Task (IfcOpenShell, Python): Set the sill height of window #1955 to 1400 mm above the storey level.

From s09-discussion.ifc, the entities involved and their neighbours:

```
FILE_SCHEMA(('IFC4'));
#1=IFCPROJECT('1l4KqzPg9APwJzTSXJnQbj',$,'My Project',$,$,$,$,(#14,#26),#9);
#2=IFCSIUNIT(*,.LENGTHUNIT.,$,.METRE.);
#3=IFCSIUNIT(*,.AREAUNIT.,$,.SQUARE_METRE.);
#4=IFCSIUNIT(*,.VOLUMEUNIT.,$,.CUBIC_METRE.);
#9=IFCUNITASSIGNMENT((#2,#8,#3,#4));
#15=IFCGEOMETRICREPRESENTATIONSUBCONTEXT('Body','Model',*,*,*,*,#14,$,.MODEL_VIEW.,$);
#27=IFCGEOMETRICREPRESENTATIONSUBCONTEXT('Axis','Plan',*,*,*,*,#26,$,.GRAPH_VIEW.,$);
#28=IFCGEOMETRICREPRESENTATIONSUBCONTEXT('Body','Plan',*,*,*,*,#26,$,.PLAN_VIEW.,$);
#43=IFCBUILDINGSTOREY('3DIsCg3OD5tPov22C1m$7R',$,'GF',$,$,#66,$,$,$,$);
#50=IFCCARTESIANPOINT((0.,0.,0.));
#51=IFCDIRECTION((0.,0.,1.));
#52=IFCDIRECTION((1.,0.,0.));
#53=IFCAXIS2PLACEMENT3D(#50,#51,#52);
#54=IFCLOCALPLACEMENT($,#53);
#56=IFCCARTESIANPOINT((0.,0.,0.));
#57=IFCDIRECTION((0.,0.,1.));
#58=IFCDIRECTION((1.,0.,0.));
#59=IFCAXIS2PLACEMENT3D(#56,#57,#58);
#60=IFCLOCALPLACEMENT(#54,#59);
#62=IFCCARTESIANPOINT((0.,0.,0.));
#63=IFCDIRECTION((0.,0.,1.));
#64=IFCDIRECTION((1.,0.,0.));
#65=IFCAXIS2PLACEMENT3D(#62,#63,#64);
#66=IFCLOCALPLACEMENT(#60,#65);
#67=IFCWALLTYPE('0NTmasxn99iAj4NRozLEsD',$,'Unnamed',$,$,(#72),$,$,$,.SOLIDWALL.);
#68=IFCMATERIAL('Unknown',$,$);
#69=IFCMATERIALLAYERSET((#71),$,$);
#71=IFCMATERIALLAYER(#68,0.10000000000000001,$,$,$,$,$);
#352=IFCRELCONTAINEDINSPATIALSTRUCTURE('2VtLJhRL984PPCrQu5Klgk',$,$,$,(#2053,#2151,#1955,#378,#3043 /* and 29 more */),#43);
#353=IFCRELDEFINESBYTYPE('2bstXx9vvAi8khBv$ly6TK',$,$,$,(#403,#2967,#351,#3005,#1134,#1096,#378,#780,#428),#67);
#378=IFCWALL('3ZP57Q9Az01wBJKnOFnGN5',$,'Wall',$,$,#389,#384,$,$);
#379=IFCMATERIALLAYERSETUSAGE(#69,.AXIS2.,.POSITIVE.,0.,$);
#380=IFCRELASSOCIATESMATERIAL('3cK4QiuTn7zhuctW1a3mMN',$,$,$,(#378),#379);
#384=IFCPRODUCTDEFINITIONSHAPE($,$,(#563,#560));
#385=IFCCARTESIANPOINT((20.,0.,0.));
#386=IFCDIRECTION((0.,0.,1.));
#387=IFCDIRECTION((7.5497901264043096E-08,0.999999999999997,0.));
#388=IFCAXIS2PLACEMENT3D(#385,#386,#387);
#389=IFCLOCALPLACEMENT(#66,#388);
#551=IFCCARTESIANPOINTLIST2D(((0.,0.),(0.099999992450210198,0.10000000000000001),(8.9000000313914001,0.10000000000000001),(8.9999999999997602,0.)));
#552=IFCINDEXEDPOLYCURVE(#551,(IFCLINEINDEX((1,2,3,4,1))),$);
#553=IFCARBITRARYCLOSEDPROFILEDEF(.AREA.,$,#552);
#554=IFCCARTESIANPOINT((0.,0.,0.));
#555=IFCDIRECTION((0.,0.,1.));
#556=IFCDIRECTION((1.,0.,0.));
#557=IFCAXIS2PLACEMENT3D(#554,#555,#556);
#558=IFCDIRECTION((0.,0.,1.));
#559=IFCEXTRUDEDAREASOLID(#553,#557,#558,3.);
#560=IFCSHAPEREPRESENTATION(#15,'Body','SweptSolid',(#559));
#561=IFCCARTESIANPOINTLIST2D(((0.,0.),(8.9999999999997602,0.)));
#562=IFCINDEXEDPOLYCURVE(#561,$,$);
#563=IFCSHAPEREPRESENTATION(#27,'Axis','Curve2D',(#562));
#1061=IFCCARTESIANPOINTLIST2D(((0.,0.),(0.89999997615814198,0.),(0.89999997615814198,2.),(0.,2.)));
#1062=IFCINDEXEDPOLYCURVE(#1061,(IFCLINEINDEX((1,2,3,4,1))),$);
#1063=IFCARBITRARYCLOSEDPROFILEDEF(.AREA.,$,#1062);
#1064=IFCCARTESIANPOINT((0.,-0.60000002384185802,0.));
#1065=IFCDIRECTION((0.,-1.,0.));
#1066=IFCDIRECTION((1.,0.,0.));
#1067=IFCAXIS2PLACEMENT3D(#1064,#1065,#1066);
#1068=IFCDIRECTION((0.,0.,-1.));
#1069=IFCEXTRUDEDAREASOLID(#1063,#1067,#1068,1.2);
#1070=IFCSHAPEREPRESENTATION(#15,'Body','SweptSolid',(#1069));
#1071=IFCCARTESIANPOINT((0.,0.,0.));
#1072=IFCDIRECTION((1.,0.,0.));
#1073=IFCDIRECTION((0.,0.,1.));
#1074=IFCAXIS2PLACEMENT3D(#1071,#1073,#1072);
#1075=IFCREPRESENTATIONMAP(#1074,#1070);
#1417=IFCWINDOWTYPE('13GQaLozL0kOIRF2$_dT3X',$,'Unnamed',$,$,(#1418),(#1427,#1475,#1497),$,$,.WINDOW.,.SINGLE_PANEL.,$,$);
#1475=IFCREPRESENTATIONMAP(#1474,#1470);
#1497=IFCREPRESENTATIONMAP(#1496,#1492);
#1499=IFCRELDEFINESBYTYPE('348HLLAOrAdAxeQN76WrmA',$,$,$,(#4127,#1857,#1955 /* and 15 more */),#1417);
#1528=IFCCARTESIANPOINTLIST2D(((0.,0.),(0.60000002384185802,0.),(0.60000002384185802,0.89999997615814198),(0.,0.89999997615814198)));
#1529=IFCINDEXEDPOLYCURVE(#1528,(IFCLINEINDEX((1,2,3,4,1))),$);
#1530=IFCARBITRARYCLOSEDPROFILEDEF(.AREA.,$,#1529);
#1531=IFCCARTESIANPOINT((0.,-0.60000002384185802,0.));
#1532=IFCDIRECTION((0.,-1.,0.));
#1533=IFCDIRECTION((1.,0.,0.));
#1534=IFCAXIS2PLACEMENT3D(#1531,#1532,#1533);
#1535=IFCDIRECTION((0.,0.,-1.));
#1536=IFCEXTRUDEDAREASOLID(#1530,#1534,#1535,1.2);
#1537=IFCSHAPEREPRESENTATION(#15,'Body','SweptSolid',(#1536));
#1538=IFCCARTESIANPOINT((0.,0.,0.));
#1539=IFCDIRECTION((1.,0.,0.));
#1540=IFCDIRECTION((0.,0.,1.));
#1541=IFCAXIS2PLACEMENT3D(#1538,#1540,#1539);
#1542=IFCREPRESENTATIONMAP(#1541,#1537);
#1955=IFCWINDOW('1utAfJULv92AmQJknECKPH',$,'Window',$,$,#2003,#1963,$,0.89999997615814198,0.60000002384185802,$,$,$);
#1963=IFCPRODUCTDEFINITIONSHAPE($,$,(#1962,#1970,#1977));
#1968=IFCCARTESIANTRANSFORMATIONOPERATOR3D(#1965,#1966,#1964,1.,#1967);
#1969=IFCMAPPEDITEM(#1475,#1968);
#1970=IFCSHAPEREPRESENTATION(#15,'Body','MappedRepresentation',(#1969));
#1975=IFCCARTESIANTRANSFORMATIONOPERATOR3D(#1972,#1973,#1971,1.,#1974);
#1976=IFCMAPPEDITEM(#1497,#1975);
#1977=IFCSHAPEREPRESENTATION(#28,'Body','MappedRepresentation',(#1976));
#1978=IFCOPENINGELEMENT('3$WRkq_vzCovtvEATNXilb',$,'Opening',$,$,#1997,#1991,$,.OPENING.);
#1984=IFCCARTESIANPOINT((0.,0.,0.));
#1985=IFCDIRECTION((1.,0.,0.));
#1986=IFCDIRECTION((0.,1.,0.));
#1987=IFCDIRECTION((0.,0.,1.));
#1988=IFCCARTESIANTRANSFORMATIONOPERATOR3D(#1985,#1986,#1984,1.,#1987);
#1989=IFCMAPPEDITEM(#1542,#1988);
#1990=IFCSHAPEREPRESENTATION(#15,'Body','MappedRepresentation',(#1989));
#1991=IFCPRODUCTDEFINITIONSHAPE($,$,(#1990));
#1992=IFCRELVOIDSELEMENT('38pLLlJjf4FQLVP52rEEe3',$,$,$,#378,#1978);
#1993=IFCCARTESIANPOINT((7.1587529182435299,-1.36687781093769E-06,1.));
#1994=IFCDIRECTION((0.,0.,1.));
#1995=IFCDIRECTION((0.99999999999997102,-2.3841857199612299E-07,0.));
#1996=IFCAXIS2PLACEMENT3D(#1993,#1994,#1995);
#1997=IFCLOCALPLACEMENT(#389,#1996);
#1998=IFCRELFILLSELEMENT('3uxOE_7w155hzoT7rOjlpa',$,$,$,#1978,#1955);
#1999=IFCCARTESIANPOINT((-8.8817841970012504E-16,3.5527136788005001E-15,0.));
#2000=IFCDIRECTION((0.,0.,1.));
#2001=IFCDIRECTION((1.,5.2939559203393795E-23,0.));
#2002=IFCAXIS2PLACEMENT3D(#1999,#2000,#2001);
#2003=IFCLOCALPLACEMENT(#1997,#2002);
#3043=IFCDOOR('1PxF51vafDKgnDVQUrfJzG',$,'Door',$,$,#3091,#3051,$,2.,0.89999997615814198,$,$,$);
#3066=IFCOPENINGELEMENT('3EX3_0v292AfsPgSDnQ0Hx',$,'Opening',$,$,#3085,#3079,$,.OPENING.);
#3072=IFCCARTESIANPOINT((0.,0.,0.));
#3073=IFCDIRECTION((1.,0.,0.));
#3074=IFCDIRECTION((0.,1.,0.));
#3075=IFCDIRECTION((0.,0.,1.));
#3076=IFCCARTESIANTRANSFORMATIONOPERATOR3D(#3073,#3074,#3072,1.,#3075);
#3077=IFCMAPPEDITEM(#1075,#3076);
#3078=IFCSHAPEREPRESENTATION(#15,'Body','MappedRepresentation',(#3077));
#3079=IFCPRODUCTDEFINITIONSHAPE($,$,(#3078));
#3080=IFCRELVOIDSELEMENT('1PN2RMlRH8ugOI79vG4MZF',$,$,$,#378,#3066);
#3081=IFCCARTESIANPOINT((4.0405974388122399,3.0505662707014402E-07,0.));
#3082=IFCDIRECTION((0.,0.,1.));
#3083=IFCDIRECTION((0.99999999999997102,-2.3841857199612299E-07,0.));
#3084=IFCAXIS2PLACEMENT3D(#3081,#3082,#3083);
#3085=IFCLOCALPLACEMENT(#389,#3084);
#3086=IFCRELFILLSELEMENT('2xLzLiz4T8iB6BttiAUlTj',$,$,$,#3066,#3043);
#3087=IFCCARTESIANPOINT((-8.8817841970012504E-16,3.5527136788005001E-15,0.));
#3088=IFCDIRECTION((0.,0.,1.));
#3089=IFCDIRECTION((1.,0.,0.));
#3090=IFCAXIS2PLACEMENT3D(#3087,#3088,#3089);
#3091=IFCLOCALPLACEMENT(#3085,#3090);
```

```python
import numpy as np
import ifcopenshell
import ifcopenshell.api.geometry
import ifcopenshell.geom
import ifcopenshell.util.element
import ifcopenshell.util.placement
import ifcopenshell.util.shape
import ifcopenshell.util.unit

model = ifcopenshell.open("s09-discussion.ifc")
unit_scale = ifcopenshell.util.unit.calculate_unit_scale(model)

window = model.by_guid("1utAfJULv92AmQJknECKPH")
opening = window.FillsVoids[0].RelatingOpeningElement
storey = ifcopenshell.util.element.get_container(window, ifc_class="IfcBuildingStorey")
level = ifcopenshell.util.placement.get_local_placement(storey.ObjectPlacement)[2, 3]

# The opening's origin need not be at the sill, so measure its lowest point.
shape = ifcopenshell.geom.create_shape(ifcopenshell.geom.settings(), opening)
bottom = ifcopenshell.util.shape.get_shape_bottom_elevation(shape, shape.geometry) / unit_scale
dz = level + 1.4 / unit_scale - bottom

shift = np.array([0.0, 0.0, dz])
# The window is placed relative to its opening, so it follows when the opening moves.
matrix = ifcopenshell.util.placement.get_local_placement(opening.ObjectPlacement)
matrix[:3, 3] += shift
ifcopenshell.api.geometry.edit_object_placement(
    model, product=opening, matrix=matrix, is_si=False, should_transform_children=True
)

print(f"moved by {dz * unit_scale:+.3f} m")

model.write("s09-discussion-out.ifc")
```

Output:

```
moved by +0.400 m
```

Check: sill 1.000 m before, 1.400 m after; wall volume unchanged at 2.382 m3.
